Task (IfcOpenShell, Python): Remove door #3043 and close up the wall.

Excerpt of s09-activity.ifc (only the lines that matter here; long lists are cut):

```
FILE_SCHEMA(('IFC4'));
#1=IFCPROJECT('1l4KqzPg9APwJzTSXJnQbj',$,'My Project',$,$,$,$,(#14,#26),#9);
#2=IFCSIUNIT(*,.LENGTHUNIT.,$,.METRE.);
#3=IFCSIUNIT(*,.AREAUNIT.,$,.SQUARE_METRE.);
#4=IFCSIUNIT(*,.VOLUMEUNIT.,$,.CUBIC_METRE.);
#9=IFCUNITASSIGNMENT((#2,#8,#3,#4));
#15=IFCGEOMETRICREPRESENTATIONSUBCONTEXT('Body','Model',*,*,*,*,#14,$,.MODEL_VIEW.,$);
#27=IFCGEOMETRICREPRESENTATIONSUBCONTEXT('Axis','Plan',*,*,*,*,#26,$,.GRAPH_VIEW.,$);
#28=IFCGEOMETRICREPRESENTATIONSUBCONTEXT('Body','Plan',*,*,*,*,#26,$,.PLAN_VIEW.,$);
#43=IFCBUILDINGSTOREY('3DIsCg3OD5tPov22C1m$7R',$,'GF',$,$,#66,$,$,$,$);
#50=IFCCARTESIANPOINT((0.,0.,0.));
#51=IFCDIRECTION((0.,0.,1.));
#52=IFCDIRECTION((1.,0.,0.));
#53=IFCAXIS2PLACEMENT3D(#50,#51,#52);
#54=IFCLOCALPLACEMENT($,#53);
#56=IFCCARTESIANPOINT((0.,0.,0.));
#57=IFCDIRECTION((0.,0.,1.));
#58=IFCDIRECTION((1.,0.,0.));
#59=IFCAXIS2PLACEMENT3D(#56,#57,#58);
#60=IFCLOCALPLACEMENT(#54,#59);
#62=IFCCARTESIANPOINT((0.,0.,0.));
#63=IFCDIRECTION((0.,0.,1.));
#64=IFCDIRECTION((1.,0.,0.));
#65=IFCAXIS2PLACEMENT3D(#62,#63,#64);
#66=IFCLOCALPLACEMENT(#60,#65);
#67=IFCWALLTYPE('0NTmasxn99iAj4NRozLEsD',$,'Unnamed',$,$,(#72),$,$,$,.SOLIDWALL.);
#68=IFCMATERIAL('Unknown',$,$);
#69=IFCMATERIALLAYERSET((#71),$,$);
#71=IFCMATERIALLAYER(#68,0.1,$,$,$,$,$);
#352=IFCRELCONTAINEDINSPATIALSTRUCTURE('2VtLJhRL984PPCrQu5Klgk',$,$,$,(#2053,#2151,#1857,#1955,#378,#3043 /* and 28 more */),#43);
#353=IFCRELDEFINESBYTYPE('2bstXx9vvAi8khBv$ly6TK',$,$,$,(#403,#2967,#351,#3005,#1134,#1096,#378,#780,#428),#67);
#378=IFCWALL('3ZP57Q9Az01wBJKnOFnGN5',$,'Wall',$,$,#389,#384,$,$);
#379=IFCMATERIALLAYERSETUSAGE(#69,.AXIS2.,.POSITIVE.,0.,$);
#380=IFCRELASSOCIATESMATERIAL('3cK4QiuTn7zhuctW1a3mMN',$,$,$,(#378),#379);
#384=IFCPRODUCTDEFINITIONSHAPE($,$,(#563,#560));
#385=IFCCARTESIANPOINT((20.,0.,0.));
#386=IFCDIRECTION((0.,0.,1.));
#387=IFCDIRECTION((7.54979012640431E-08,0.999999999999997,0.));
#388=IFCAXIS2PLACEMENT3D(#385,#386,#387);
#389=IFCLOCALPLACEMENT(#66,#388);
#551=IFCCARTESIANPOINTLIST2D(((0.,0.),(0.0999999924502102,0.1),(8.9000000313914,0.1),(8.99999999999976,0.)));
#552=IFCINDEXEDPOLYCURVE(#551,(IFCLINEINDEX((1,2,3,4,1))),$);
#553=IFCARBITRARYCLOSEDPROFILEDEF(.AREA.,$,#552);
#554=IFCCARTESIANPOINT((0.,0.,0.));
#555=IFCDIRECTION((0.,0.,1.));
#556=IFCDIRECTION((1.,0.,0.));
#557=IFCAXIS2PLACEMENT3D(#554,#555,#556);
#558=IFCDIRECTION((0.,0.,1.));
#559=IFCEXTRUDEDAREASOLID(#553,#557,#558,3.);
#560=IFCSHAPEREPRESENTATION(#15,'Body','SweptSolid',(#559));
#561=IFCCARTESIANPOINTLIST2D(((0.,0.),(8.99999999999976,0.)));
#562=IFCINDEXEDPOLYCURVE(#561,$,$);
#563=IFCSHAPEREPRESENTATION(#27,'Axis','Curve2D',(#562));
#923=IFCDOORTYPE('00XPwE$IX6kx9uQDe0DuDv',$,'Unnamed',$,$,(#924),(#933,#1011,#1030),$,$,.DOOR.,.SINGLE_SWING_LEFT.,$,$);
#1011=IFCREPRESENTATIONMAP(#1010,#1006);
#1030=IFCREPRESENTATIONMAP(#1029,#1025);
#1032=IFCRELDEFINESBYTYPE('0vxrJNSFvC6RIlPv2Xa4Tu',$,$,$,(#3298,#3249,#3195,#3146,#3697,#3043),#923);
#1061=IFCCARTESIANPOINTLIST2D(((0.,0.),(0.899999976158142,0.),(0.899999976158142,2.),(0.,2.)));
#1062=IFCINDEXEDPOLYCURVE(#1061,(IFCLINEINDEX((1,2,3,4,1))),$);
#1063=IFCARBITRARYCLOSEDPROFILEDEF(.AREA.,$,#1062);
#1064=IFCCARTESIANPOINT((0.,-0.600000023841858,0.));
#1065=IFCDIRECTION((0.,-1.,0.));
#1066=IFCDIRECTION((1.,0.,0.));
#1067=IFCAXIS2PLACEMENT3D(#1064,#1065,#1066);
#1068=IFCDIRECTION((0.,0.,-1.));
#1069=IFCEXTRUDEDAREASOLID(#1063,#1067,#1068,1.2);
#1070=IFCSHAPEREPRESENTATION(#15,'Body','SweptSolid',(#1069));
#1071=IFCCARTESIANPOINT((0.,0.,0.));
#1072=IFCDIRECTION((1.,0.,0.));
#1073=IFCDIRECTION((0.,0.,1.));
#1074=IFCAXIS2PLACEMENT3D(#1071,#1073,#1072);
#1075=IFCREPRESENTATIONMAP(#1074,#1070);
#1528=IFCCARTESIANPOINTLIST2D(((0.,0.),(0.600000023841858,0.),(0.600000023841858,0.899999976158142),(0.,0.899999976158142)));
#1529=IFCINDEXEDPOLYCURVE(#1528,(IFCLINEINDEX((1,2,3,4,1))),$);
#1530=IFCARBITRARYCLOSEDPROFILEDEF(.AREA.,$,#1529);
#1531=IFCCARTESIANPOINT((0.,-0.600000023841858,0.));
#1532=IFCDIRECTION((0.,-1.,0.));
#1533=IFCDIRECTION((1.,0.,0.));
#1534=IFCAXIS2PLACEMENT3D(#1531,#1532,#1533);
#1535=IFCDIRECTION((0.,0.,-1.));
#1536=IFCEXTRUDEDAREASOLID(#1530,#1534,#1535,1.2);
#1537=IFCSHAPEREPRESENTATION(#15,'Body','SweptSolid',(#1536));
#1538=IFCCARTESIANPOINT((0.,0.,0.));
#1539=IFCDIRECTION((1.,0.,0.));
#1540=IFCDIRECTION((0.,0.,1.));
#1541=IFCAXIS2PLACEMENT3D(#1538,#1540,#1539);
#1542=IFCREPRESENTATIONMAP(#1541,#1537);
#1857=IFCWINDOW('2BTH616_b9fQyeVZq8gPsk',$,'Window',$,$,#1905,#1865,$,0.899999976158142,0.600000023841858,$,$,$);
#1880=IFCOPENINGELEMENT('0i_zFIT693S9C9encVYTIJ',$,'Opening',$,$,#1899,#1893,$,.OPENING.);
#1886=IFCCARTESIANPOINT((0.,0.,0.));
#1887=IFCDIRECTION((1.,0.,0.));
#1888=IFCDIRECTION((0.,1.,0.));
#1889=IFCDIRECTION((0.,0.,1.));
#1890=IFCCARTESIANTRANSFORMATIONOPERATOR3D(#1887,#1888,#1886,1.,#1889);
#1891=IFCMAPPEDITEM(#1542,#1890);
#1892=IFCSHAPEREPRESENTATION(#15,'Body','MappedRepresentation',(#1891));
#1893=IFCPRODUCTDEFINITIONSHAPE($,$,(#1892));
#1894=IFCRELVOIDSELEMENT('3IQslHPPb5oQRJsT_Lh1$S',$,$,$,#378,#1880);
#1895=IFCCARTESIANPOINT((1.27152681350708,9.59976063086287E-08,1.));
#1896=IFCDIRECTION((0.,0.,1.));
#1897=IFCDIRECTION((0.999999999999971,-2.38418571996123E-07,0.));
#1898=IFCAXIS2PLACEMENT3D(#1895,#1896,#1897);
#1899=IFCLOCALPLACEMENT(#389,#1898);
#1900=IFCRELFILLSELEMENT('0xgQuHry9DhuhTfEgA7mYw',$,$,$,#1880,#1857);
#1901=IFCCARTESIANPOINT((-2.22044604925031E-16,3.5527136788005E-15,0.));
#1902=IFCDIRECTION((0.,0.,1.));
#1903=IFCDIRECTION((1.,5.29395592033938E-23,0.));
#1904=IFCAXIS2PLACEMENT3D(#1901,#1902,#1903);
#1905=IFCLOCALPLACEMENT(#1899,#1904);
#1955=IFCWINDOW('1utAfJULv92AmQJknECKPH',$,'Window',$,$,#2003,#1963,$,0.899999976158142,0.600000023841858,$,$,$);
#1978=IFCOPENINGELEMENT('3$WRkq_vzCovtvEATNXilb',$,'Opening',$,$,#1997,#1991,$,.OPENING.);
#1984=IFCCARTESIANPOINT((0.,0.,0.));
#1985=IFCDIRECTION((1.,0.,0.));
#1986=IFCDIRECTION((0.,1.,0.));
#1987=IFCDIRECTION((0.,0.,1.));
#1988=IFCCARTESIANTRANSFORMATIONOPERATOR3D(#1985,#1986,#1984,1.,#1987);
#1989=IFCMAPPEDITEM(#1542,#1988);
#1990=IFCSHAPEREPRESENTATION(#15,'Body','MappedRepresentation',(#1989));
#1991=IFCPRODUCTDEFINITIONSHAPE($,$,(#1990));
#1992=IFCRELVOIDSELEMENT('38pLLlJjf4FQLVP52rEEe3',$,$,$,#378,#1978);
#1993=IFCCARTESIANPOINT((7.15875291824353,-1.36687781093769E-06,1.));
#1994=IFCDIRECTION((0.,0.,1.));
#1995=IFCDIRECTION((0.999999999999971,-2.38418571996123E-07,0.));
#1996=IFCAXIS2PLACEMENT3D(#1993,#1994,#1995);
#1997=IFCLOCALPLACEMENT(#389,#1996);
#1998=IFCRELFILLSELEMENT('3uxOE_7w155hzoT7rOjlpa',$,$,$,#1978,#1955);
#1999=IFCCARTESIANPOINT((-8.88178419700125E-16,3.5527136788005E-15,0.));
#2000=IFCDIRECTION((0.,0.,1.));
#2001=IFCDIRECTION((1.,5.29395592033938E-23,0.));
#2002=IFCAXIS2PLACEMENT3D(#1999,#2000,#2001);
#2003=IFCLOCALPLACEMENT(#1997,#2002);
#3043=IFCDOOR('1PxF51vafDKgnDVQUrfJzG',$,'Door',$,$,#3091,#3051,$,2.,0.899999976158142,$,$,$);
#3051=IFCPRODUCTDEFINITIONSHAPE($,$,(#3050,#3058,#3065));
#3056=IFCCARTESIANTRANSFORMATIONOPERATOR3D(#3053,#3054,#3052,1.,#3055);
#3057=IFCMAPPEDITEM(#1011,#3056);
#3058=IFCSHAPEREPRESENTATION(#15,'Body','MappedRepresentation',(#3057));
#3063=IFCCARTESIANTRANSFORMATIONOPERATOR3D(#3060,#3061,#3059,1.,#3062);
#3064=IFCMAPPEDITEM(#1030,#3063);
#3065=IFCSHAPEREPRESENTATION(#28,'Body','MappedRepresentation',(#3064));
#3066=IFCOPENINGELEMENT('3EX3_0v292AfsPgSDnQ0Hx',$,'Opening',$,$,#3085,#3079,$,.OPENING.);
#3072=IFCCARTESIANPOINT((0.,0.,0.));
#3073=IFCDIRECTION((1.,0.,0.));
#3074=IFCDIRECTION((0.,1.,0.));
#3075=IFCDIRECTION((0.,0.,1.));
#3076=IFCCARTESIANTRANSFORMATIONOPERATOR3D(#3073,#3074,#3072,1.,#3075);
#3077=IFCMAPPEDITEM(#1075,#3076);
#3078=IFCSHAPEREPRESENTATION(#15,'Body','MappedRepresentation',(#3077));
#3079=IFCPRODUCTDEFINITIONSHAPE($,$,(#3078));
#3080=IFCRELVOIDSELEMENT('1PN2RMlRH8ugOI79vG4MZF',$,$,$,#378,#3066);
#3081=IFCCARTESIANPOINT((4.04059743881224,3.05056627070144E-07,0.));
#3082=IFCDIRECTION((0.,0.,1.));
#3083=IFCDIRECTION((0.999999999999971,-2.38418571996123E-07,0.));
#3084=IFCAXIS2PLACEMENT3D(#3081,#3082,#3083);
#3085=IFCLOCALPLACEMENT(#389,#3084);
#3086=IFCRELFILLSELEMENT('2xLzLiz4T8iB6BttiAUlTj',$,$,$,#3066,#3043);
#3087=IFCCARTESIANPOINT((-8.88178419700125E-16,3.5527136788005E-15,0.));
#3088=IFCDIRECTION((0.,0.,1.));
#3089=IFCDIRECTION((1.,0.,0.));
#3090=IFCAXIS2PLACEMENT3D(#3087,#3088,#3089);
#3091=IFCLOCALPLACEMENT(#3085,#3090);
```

```python
import ifcopenshell
import ifcopenshell.api.feature
import ifcopenshell.api.root
import ifcopenshell.geom
import ifcopenshell.util.shape

model = ifcopenshell.open("s09-activity.ifc")
settings = ifcopenshell.geom.settings()


def volume(element):
    """Net volume in cubic metres, openings subtracted."""
    shape = ifcopenshell.geom.create_shape(settings, element)
    return ifcopenshell.util.shape.get_volume(shape.geometry)


door = model.by_id(3043)
opening = door.FillsVoids[0].RelatingOpeningElement
wall = opening.VoidsElements[0].RelatingBuildingElement
before = volume(wall)

ifcopenshell.api.root.remove_product(model, product=door)
ifcopenshell.api.feature.remove_feature(model, feature=opening)

after = volume(wall)

print(f"wall volume {before:.3f} -> {after:.3f} m3")

model.write("s09-activity-out.ifc")
```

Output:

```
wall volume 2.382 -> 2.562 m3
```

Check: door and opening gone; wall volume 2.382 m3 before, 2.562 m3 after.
